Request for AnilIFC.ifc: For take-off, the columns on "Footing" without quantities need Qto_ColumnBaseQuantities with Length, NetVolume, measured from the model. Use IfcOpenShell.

First a look at what the model holds.

```python
import ifcopenshell
import ifcopenshell.util.element
import ifcopenshell.util.unit

model = ifcopenshell.open("AnilIFC.ifc")
print(model.schema)
for unit_type in ("LENGTHUNIT", "AREAUNIT", "VOLUMEUNIT"):
    print(unit_type, ifcopenshell.util.unit.calculate_unit_scale(model, unit_type))
storey = next(s for s in model.by_type("IfcBuildingStorey") if s.Name == "Footing")
columns = [e for e in ifcopenshell.util.element.get_decomposition(storey) if e.is_a("IfcColumn")]
for e in sorted(columns, key=lambda e: e.id()):
    print(e.id(), e.is_a(), e.Name, list(ifcopenshell.util.element.get_psets(e, qtos_only=True)), sep=" | ")
```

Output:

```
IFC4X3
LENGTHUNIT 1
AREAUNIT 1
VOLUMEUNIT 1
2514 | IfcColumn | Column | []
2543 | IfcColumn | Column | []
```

```python
import ifcopenshell
import ifcopenshell.api.pset
import ifcopenshell.geom
import ifcopenshell.util.element
import ifcopenshell.util.shape
import ifcopenshell.util.unit

model = ifcopenshell.open("AnilIFC.ifc")
unit_scale = ifcopenshell.util.unit.calculate_unit_scale(model)
volume_scale = ifcopenshell.util.unit.calculate_unit_scale(model, "VOLUMEUNIT")
settings = ifcopenshell.geom.settings()

storey = next(s for s in model.by_type("IfcBuildingStorey") if s.Name == "Footing")
columns = [e for e in ifcopenshell.util.element.get_decomposition(storey) if e.is_a("IfcColumn")]

for e in sorted(columns, key=lambda e: e.id()):
    if ifcopenshell.util.element.get_psets(e, qtos_only=True, should_inherit=False):
        continue
    # Geometry comes back in metres, in the element's own axes.
    shape = ifcopenshell.geom.create_shape(settings, e)
    values = {
        "Length": ifcopenshell.util.shape.get_z(shape.geometry) / unit_scale,
        "NetVolume": ifcopenshell.util.shape.get_volume(shape.geometry) / volume_scale,
    }
    qto = ifcopenshell.api.pset.add_qto(model, product=e, name="Qto_ColumnBaseQuantities")
    ifcopenshell.api.pset.edit_qto(model, qto=qto, properties=values)
    print(e.id(), {k: round(v, 3) for k, v in values.items()})

model.write("AnilIFC-out.ifc")
```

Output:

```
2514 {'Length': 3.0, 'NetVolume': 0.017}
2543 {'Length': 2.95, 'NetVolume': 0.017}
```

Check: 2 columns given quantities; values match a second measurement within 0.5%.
